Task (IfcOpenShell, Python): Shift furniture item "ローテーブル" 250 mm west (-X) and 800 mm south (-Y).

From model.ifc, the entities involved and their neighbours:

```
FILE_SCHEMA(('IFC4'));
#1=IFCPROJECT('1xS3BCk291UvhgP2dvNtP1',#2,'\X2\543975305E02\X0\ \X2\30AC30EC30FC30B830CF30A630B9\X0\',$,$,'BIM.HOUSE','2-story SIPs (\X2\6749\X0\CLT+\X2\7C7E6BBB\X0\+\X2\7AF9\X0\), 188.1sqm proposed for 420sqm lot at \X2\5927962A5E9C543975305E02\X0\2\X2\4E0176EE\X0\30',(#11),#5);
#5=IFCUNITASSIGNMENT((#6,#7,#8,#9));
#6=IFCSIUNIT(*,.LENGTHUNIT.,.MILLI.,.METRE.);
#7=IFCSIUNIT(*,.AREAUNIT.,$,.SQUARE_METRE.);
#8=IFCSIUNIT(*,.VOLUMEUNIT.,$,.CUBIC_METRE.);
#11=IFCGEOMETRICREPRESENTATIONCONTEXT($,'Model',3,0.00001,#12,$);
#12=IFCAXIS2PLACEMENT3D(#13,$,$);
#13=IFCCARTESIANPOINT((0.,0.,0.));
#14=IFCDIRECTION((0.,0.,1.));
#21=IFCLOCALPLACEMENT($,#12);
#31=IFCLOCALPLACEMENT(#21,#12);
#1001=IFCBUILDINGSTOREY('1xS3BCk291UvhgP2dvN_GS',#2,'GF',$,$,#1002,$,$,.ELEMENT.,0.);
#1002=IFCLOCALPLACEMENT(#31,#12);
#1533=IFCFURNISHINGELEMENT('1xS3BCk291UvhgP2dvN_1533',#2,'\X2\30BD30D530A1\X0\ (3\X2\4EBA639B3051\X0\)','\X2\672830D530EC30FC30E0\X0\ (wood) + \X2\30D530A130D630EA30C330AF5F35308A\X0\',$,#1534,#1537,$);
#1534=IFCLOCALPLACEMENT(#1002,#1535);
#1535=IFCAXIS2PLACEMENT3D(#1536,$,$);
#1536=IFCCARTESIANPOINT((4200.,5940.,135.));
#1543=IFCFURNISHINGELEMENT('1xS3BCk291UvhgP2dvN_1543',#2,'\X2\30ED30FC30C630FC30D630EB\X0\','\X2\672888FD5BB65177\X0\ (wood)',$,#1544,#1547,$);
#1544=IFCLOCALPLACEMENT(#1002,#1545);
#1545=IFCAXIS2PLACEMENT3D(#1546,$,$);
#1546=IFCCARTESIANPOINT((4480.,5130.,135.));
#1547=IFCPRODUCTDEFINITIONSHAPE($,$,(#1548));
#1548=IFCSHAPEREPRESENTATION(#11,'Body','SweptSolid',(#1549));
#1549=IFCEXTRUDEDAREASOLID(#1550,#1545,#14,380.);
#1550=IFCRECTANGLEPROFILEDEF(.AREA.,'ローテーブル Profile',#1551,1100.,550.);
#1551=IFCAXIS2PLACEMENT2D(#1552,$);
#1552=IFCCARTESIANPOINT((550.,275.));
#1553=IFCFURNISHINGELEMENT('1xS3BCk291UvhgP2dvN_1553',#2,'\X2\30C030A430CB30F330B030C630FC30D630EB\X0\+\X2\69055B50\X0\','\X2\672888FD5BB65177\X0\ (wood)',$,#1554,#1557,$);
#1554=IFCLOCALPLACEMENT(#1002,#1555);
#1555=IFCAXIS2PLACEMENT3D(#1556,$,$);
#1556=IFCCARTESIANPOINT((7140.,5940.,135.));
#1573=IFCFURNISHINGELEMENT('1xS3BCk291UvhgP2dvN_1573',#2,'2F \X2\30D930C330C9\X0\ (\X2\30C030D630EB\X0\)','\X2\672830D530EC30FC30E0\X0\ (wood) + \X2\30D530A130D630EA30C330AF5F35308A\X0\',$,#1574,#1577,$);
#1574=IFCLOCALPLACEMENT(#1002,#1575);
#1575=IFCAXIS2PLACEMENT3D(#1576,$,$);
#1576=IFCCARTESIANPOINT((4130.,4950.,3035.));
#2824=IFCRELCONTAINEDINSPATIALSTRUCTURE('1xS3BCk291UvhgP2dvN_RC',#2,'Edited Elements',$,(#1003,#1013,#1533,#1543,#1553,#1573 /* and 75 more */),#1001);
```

```python
import ifcopenshell
import ifcopenshell.api.geometry
import ifcopenshell.util.placement

model = ifcopenshell.open("model.ifc")

item = model.by_id(1543)
matrix = ifcopenshell.util.placement.get_local_placement(item.ObjectPlacement)
matrix[0, 3] -= 250.0
matrix[1, 3] -= 800.0
ifcopenshell.api.geometry.edit_object_placement(model, product=item, matrix=matrix, is_si=False)

print(ifcopenshell.util.placement.get_local_placement(item.ObjectPlacement).round(3) + 0.0)

model.write("model_edited.ifc")
```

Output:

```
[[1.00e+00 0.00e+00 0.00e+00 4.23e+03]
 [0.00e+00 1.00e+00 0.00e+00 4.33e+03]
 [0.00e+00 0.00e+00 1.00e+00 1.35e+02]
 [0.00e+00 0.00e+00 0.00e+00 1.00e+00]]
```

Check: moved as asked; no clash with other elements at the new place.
